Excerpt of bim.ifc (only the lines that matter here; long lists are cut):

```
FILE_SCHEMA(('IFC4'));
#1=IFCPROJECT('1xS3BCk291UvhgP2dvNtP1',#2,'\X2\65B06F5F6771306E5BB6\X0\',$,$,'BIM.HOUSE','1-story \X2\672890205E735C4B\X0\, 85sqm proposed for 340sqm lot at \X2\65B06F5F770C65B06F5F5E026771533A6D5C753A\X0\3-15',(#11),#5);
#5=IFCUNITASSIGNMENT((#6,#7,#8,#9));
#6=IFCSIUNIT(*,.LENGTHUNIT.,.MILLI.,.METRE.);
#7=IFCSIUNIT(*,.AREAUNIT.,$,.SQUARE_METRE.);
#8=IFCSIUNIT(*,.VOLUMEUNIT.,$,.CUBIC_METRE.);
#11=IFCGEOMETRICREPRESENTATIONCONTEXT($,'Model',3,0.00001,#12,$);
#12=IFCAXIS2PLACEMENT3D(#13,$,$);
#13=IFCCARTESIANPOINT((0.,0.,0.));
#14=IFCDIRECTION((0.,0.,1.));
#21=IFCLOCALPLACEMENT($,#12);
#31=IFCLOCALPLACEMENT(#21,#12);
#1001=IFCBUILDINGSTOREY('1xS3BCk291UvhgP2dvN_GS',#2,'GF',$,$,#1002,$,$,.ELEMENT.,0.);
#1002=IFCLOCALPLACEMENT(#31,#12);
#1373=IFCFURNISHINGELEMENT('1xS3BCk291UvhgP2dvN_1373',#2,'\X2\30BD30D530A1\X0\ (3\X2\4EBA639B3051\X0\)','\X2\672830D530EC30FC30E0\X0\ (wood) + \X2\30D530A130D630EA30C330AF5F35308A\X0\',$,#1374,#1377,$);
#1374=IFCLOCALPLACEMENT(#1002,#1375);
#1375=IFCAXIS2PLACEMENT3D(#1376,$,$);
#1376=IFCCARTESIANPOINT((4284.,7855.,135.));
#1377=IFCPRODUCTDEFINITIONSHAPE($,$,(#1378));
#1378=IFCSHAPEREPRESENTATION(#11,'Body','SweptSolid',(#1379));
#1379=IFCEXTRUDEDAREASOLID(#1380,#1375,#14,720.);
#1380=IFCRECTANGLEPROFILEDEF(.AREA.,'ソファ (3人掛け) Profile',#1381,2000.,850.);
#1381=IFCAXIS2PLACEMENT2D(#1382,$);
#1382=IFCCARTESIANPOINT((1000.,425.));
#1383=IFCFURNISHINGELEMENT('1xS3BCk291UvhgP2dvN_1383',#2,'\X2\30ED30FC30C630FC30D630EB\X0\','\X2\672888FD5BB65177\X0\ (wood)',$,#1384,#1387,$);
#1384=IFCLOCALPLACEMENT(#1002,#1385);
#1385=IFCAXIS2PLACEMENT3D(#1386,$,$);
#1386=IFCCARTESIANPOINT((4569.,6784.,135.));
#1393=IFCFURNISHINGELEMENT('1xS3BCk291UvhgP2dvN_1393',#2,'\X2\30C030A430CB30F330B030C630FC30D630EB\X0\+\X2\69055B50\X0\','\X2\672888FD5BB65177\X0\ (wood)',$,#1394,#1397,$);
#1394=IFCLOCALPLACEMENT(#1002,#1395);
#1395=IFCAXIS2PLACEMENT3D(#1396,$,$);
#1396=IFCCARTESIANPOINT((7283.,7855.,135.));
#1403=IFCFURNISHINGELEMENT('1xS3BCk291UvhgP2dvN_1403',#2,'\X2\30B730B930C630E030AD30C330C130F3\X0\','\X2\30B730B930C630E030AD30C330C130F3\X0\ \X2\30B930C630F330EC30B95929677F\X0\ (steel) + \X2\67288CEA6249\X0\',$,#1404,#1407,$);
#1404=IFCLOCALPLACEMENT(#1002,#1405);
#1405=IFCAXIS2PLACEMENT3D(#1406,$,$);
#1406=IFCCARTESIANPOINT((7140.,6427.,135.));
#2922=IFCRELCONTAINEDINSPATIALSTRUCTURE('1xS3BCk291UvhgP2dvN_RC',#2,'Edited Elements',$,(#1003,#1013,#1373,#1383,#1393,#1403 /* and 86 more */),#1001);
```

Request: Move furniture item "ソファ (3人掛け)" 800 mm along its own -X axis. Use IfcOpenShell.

```python
import ifcopenshell
import ifcopenshell.api.geometry
import ifcopenshell.util.placement
import ifcopenshell.util.unit

model = ifcopenshell.open("bim.ifc")
unit_scale = ifcopenshell.util.unit.calculate_unit_scale(model)

item = model.by_guid("1xS3BCk291UvhgP2dvN_1373")
matrix = ifcopenshell.util.placement.get_local_placement(item.ObjectPlacement)
matrix[:3, 3] -= matrix[:3, 0] * 0.8 / unit_scale
ifcopenshell.api.geometry.edit_object_placement(model, product=item, matrix=matrix, is_si=False)

print(ifcopenshell.util.placement.get_local_placement(item.ObjectPlacement).round(3) + 0.0)

model.write("bim_rev.ifc")
```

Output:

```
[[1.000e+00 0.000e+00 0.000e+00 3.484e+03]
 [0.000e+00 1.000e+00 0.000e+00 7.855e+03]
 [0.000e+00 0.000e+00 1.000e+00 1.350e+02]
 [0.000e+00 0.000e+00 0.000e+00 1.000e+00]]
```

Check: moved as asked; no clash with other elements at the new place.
